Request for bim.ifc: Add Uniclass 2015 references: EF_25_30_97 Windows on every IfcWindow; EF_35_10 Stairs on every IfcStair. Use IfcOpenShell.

First a look at what the model holds.

```python
import ifcopenshell

model = ifcopenshell.open("bim.ifc")
print(model.schema)
print("classifications:", [c.Name for c in model.by_type("IfcClassification")])
for ifc_class in ("IfcDoor", "IfcRoof", "IfcStair", "IfcWall", "IfcWindow"):
    print(ifc_class, len(model.by_type(ifc_class)))
```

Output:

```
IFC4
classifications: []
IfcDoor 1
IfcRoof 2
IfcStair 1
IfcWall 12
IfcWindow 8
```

```python
import ifcopenshell
import ifcopenshell.api.classification

model = ifcopenshell.open("bim.ifc")

system = ifcopenshell.api.classification.add_classification(model, classification="Uniclass 2015")

codes = {
    "IfcWindow": ("EF_25_30_97", "Windows"),
    "IfcStair": ("EF_35_10", "Stairs"),
}
for ifc_class, (code, name) in codes.items():
    products = model.by_type(ifc_class)
    ifcopenshell.api.classification.add_reference(
        model, products=products, classification=system, identification=code, name=name
    )
    print(code, len(products))

model.write("bim_updated.ifc")
```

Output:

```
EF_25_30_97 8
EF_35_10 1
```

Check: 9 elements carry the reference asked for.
